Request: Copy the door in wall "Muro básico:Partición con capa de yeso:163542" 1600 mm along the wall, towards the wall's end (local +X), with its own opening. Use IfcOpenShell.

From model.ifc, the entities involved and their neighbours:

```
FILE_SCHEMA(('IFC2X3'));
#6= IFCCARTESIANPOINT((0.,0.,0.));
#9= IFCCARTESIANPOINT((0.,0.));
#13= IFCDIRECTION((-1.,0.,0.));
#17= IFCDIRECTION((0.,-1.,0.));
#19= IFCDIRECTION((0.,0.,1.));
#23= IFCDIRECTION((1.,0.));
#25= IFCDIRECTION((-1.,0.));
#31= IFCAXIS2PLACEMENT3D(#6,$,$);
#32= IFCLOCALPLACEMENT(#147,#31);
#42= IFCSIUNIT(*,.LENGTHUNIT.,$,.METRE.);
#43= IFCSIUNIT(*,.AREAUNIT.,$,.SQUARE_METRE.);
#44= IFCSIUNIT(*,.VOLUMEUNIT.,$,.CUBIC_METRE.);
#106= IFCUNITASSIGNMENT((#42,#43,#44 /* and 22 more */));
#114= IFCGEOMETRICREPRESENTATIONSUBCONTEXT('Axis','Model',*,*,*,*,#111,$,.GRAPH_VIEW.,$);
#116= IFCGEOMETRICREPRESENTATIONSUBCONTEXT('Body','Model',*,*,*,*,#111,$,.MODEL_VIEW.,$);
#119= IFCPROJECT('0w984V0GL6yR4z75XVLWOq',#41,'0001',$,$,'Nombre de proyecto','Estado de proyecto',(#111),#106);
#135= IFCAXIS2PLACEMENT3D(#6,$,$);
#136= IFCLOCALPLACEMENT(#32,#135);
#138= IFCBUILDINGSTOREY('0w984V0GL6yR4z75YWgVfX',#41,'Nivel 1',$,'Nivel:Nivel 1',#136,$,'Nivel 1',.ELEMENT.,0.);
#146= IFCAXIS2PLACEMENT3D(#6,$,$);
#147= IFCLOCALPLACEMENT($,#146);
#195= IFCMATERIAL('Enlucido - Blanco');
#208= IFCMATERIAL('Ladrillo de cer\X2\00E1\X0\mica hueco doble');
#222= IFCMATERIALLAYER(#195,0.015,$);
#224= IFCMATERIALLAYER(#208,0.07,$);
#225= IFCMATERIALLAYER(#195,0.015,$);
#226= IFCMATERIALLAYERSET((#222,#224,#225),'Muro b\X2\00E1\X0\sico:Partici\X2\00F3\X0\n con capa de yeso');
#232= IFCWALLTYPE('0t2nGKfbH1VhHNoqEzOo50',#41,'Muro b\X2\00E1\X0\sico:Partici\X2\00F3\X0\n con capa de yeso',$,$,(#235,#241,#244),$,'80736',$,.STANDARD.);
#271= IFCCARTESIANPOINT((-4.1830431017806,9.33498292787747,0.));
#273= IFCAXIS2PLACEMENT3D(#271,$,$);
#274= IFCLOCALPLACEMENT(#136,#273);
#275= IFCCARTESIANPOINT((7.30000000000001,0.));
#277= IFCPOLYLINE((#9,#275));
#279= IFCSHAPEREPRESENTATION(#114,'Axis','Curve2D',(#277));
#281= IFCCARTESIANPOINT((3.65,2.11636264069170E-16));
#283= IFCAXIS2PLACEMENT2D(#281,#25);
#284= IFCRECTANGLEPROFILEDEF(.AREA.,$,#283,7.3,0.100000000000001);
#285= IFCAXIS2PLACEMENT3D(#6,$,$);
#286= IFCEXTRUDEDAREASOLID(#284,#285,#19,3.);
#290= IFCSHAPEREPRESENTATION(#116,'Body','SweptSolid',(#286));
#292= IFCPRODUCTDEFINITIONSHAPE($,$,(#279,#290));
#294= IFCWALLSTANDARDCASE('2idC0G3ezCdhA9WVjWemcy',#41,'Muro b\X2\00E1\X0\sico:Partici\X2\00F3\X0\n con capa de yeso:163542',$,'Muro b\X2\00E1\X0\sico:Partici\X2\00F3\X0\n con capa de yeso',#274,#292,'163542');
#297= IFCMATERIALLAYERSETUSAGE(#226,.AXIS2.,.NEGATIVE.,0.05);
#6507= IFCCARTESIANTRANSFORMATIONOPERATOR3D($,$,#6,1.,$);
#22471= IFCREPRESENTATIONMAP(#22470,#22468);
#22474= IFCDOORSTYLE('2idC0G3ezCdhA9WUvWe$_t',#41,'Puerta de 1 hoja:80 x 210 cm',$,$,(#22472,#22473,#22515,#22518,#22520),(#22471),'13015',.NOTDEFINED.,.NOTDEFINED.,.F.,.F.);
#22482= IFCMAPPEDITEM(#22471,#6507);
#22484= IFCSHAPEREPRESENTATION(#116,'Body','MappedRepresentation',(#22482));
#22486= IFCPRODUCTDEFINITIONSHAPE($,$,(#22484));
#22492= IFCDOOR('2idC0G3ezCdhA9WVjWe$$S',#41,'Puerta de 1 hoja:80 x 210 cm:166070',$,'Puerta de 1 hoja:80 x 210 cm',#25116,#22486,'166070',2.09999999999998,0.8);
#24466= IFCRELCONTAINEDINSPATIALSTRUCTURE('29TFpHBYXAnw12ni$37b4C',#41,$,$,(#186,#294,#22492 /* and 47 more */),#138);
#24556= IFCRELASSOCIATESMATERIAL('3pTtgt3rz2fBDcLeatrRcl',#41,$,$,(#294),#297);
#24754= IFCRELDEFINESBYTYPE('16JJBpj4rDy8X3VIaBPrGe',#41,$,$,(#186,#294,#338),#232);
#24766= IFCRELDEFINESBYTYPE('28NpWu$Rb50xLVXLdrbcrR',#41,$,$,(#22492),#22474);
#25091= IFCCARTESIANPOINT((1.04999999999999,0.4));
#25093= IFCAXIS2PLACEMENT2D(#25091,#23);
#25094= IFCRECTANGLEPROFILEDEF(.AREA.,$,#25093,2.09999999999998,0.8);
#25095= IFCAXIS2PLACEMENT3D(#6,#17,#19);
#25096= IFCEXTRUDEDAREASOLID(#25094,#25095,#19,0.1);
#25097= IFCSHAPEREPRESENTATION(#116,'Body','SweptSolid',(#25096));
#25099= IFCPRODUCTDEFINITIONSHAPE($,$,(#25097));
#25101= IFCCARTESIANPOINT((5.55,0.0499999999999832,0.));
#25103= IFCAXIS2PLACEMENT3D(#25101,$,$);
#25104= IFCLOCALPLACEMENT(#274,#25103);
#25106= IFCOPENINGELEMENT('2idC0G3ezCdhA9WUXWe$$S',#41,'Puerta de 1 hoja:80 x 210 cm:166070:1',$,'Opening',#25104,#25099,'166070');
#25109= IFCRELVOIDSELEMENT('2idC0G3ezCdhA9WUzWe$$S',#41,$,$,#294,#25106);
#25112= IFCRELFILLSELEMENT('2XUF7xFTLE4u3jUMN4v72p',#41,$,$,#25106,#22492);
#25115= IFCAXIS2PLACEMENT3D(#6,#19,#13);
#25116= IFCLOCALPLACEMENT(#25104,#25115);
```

```python
import ifcopenshell
import ifcopenshell.api.feature
import ifcopenshell.api.geometry
import ifcopenshell.api.root
import ifcopenshell.geom
import ifcopenshell.util.element
import ifcopenshell.util.placement
import ifcopenshell.util.shape

model = ifcopenshell.open("model.ifc")
settings = ifcopenshell.geom.settings()


def volume(element):
    """Net volume in cubic metres, openings subtracted."""
    shape = ifcopenshell.geom.create_shape(settings, element)
    return ifcopenshell.util.shape.get_volume(shape.geometry)


def reuse_history(source, copy):
    """copy_class also copies each property set's owner history, people and application; keep the originals."""
    for rel in copy.IsDefinedBy:
        if rel.is_a("IfcRelDefinesByProperties") and (history := rel.RelatingPropertyDefinition.OwnerHistory):
            rel.RelatingPropertyDefinition.OwnerHistory = source.OwnerHistory
            ifcopenshell.util.element.remove_deep2(model, history)


door = model.by_guid("2idC0G3ezCdhA9WVjWe$$S")
opening = door.FillsVoids[0].RelatingOpeningElement
wall = opening.VoidsElements[0].RelatingBuildingElement
before = volume(wall)
shift = ifcopenshell.util.placement.get_local_placement(wall.ObjectPlacement)[:3, 0] * 1.6

# copy_class copies the void relationship, type, container and properties, but no geometry.
new_opening = ifcopenshell.api.root.copy_class(model, product=opening)
new_opening.Representation = ifcopenshell.util.element.copy_deep(
    model, opening.Representation, exclude=["IfcGeometricRepresentationContext", "IfcRepresentationMap"]
)
new_opening.Name = "Puerta de 1 hoja:80 x 210 cm"
new_opening.Tag = None
new_door = ifcopenshell.api.root.copy_class(model, product=door)
new_door.Representation = ifcopenshell.util.element.copy_deep(
    model, door.Representation, exclude=["IfcGeometricRepresentationContext", "IfcRepresentationMap"]
)
new_door.Name = "Puerta de 1 hoja:80 x 210 cm"
new_door.Tag = None
reuse_history(door, new_door)
fills = ifcopenshell.api.feature.add_filling(model, opening=new_opening, element=new_door)
fills.OwnerHistory = new_door.OwnerHistory  # required in IFC2X3

for old, new in ((opening, new_opening), (door, new_door)):
    matrix = ifcopenshell.util.placement.get_local_placement(old.ObjectPlacement)
    matrix[:3, 3] += shift
    ifcopenshell.api.geometry.edit_object_placement(model, product=new, matrix=matrix, is_si=False)

after = volume(wall)

print(f"wall volume {before:.3f} -> {after:.3f} m3")

model.write("model_edited.ifc")
```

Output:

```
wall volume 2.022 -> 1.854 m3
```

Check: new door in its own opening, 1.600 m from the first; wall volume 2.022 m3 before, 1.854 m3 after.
